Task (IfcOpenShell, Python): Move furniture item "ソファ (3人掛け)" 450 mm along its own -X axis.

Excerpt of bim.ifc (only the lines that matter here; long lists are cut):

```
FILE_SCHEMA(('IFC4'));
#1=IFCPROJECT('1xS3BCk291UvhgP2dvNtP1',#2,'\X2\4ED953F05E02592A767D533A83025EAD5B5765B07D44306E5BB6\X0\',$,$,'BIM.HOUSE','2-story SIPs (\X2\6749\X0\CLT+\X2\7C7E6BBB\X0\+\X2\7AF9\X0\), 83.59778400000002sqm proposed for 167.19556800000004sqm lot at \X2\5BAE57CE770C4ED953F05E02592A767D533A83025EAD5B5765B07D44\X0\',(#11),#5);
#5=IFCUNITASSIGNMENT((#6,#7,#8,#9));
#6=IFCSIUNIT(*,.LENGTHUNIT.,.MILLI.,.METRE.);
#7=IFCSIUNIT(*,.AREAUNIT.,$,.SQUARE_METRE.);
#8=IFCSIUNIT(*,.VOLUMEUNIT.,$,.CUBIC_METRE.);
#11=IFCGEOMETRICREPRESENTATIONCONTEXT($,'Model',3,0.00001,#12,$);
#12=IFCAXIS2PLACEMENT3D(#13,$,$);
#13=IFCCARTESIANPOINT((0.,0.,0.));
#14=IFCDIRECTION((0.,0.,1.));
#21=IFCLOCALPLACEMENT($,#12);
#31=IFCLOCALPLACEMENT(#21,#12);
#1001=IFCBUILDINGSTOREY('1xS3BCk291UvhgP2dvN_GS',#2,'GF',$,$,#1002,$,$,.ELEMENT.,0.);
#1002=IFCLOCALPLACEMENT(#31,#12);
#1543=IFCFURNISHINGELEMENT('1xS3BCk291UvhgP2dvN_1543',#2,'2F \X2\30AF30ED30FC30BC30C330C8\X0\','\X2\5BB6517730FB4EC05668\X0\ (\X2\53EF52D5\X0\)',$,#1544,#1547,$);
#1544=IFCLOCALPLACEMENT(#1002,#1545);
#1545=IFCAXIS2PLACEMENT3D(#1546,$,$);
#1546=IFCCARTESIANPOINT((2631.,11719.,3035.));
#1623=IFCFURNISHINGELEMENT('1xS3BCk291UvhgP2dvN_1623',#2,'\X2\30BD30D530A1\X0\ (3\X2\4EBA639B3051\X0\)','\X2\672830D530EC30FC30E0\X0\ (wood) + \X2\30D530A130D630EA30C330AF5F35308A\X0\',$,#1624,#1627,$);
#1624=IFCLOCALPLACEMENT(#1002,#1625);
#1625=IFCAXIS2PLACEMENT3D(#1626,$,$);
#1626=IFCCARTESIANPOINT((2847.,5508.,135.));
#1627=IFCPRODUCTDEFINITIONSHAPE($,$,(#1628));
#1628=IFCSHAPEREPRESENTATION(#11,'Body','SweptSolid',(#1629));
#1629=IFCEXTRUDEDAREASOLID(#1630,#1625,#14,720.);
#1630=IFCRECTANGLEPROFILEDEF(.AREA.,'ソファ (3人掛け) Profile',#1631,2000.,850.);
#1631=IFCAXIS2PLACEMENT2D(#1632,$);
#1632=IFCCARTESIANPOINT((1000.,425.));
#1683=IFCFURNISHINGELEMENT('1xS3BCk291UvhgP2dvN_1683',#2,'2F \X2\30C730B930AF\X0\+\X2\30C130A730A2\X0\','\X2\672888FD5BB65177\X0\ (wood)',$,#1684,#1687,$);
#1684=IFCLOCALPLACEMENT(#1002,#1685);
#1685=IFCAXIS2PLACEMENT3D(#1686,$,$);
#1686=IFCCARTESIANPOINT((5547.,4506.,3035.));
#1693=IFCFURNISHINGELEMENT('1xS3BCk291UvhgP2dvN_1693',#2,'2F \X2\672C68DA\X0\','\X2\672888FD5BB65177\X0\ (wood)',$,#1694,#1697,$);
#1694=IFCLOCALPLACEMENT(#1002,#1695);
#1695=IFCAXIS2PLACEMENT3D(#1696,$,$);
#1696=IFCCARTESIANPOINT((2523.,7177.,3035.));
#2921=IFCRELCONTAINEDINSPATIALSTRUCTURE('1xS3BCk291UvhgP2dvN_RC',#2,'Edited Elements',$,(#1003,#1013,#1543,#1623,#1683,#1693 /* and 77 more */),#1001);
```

```python
import ifcopenshell
import ifcopenshell.api.geometry
import ifcopenshell.util.placement

model = ifcopenshell.open("bim.ifc")

item = model.by_guid("1xS3BCk291UvhgP2dvN_1623")
matrix = ifcopenshell.util.placement.get_local_placement(item.ObjectPlacement)
matrix[:3, 3] -= matrix[:3, 0] * 450.0
ifcopenshell.api.geometry.edit_object_placement(model, product=item, matrix=matrix, is_si=False)

print(ifcopenshell.util.placement.get_local_placement(item.ObjectPlacement).round(3) + 0.0)

model.write("bim_v2.ifc")
```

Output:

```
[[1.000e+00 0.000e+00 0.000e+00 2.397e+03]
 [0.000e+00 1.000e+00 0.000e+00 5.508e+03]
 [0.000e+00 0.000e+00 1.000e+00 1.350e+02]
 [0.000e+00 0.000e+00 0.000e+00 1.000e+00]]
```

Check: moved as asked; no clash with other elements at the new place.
